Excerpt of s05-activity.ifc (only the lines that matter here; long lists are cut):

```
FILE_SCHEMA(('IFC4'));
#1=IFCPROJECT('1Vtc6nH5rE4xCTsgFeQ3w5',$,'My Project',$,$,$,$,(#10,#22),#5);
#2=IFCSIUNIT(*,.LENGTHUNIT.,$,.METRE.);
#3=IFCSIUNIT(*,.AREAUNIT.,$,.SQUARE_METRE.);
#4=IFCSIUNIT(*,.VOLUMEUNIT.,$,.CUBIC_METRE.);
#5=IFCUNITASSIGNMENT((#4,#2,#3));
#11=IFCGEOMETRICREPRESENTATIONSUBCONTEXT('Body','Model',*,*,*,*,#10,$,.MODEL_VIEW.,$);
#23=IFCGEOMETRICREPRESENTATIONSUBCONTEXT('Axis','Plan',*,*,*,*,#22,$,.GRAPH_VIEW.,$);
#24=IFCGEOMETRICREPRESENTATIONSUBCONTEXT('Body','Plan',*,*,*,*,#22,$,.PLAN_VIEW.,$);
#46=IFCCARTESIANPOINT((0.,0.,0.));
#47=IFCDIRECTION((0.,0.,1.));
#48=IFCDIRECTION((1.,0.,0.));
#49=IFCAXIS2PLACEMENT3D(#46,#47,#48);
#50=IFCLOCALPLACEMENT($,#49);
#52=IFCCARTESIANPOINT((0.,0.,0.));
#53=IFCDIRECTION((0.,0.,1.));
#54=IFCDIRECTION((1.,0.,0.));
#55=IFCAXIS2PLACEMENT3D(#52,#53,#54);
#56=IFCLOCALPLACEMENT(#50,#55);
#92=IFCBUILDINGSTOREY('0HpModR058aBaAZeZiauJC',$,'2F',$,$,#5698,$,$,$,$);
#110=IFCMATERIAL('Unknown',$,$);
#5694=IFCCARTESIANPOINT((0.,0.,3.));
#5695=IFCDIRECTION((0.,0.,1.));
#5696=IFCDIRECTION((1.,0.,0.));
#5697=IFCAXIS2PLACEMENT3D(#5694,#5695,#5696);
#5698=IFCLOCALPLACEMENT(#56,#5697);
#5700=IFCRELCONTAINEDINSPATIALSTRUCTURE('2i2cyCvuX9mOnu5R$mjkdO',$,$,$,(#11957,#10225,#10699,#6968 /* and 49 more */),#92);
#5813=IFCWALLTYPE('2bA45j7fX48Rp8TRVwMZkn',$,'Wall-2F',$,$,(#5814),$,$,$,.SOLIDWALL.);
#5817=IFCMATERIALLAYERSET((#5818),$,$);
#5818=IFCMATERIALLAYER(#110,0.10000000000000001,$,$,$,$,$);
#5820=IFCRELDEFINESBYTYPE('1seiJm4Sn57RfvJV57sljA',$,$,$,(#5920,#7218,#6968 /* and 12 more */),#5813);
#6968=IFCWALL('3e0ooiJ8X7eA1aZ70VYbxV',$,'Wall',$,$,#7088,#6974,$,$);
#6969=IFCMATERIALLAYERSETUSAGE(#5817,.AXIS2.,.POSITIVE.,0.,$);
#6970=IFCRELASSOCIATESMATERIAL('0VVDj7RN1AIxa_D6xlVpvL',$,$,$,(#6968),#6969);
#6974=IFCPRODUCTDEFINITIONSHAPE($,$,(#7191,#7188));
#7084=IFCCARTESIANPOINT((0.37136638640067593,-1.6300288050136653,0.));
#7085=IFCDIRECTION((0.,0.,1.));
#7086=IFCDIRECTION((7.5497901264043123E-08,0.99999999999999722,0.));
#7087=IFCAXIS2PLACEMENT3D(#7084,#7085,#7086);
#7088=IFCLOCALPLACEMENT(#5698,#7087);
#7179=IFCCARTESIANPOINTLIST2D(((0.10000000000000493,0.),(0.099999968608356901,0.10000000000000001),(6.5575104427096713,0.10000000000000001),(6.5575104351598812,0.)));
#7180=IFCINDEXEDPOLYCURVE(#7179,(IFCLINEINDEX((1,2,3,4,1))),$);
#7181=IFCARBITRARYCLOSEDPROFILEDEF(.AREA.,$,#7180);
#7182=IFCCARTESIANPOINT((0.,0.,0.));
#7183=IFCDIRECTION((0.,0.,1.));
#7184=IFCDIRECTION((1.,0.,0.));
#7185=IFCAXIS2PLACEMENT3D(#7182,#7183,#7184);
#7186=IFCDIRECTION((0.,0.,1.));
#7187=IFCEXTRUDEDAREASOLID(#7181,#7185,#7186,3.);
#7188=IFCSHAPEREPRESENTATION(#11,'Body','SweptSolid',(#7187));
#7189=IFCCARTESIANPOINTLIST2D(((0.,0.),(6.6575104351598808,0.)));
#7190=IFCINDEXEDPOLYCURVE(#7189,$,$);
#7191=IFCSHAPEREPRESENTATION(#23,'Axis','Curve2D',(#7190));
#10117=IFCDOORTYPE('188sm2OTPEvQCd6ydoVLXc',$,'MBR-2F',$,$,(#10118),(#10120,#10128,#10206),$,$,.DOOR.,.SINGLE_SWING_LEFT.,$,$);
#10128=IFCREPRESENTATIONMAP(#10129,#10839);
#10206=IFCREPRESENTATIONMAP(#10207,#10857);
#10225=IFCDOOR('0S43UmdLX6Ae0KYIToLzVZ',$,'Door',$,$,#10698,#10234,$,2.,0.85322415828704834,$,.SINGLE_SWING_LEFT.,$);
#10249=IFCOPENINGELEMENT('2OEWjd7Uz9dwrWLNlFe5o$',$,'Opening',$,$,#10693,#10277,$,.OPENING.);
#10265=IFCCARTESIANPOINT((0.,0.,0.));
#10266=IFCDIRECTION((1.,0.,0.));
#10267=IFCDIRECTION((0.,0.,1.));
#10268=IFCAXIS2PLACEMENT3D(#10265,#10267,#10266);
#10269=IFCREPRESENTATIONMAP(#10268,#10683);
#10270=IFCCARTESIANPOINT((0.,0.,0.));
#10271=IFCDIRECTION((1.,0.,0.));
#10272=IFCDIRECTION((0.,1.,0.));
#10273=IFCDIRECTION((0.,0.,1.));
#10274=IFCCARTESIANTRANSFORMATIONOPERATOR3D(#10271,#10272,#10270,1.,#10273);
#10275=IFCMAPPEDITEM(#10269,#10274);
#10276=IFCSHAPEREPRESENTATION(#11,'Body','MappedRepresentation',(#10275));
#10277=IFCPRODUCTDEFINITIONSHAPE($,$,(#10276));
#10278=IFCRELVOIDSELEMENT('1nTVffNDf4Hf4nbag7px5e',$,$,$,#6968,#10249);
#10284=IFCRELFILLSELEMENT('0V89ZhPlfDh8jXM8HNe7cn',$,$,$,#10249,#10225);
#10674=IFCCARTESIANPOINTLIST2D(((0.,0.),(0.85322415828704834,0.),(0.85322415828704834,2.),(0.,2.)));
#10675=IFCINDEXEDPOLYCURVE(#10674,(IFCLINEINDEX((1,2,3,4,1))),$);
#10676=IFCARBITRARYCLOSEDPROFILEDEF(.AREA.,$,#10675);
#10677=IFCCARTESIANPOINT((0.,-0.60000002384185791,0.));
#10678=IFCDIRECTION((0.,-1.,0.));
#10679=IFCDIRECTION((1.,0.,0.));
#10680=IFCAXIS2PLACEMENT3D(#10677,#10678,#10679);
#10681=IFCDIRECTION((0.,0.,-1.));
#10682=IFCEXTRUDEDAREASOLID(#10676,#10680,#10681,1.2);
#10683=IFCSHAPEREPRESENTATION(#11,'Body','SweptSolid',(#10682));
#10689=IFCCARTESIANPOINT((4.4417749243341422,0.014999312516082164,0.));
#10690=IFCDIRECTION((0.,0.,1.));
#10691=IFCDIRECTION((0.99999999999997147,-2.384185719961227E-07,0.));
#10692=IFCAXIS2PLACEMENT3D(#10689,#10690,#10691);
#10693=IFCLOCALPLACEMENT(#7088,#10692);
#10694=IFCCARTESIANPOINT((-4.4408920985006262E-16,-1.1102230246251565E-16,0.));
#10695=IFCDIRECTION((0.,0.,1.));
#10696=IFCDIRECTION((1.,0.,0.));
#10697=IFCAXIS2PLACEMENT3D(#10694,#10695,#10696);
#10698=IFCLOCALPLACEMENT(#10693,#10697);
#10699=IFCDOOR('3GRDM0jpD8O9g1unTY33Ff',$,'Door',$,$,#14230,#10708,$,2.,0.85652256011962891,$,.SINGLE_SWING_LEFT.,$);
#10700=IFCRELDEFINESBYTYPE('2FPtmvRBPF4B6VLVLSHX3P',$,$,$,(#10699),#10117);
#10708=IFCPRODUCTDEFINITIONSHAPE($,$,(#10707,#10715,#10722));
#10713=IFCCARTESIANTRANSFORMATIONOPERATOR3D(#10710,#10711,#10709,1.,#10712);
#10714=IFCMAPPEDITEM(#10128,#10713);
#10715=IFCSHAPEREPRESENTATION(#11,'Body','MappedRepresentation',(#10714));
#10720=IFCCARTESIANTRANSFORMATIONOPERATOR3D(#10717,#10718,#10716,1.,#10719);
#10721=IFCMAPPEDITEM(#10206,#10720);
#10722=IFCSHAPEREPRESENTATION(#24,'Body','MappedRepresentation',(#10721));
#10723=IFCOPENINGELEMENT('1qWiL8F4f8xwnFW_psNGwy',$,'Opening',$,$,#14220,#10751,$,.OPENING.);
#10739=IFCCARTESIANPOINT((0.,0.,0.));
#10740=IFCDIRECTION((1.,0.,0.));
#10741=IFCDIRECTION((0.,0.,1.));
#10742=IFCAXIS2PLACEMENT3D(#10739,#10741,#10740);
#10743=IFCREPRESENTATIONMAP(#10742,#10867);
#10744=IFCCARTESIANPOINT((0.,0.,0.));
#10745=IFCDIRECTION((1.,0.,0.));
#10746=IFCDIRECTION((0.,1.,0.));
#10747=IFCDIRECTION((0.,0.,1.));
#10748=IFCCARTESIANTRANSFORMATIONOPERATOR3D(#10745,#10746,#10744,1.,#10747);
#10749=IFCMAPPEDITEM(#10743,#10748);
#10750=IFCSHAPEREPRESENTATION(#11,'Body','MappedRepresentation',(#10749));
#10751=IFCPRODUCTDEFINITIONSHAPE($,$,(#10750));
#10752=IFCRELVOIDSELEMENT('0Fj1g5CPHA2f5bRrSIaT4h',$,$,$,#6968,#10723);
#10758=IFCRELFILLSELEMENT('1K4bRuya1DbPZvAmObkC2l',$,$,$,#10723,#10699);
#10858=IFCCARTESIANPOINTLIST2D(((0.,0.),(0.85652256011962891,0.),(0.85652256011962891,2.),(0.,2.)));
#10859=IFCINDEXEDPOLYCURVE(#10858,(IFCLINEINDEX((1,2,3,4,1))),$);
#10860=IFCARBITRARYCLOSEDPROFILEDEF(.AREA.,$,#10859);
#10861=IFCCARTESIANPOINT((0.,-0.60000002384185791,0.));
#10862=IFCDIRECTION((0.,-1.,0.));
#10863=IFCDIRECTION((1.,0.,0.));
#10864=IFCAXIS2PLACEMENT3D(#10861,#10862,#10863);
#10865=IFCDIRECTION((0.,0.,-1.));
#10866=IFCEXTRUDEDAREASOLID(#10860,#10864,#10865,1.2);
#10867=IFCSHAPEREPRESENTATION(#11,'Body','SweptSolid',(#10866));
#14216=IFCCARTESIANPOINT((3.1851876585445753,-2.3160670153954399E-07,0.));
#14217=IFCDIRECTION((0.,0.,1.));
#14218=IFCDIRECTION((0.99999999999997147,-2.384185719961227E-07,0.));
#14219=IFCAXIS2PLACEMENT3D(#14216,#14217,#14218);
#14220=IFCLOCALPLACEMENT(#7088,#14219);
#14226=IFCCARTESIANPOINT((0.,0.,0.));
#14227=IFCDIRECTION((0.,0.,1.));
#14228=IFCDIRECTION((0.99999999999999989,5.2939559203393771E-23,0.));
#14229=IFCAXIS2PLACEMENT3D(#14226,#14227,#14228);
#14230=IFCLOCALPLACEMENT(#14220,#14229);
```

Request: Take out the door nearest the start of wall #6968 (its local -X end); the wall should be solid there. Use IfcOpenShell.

```python
import ifcopenshell
import ifcopenshell.api.feature
import ifcopenshell.api.root
import ifcopenshell.geom
import ifcopenshell.util.shape

model = ifcopenshell.open("s05-activity.ifc")
settings = ifcopenshell.geom.settings()


def volume(element):
    """Net volume in cubic metres, openings subtracted."""
    shape = ifcopenshell.geom.create_shape(settings, element)
    return ifcopenshell.util.shape.get_volume(shape.geometry)


door = model.by_guid("3GRDM0jpD8O9g1unTY33Ff")
opening = door.FillsVoids[0].RelatingOpeningElement
wall = opening.VoidsElements[0].RelatingBuildingElement
before = volume(wall)

ifcopenshell.api.root.remove_product(model, product=door)
ifcopenshell.api.feature.remove_feature(model, feature=opening)

after = volume(wall)

print(f"wall volume {before:.3f} -> {after:.3f} m3")

model.write("s05-activity_edited.ifc")
```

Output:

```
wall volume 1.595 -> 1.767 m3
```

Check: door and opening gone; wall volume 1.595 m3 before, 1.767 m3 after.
